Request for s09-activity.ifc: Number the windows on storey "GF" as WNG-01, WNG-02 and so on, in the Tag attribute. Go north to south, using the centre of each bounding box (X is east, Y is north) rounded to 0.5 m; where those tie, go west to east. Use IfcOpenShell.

First a look at what the model holds.

```python
import ifcopenshell
import ifcopenshell.util.element
import ifcopenshell.util.placement

model = ifcopenshell.open("s09-activity.ifc")
print(model.schema)
storey = next(s for s in model.by_type("IfcBuildingStorey") if s.Name == "GF")
windows = [e for e in ifcopenshell.util.element.get_decomposition(storey) if e.is_a("IfcWindow")]
for e in sorted(windows, key=lambda e: e.id()):
    origin = ifcopenshell.util.placement.get_local_placement(e.ObjectPlacement)[:3, 3]
    print(e.id(), e.Tag, e.Name, origin.round(2) + 0.0, sep=" | ")
```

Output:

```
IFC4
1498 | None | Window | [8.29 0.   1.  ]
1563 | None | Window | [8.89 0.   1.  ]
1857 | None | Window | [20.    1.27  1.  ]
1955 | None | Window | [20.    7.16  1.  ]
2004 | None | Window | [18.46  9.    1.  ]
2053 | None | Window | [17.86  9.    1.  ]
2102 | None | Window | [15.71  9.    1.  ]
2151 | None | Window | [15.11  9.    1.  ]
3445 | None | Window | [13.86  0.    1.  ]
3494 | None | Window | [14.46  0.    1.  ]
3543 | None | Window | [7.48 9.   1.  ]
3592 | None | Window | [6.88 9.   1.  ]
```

```python
import ifcopenshell
import ifcopenshell.geom
import ifcopenshell.util.element
import ifcopenshell.util.shape

model = ifcopenshell.open("s09-activity.ifc")
settings = ifcopenshell.geom.settings()
settings.set("use-world-coords", True)


def centre(element):
    shape = ifcopenshell.geom.create_shape(settings, element)
    return ifcopenshell.util.shape.get_bbox_centroid(shape.geometry)


storey = next(s for s in model.by_type("IfcBuildingStorey") if s.Name == "GF")
windows = [e for e in ifcopenshell.util.element.get_decomposition(storey) if e.is_a("IfcWindow")]

# Insertion points can sit at a corner or the storey origin, so sort by the geometry (in metres).
centres = {e: centre(e) for e in windows}
windows.sort(key=lambda e: (-round(centres[e][1] / 0.5), centres[e][0]))

for i, e in enumerate(windows, start=1):
    number = f"WNG-{i:02d}"
    e.Tag = number
    print(e.id(), number)

model.write("s09-activity_edited.ifc")
```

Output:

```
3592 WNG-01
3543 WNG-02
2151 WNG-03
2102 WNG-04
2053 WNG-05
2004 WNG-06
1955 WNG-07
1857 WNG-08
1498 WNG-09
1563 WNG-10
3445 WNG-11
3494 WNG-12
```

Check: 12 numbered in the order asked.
